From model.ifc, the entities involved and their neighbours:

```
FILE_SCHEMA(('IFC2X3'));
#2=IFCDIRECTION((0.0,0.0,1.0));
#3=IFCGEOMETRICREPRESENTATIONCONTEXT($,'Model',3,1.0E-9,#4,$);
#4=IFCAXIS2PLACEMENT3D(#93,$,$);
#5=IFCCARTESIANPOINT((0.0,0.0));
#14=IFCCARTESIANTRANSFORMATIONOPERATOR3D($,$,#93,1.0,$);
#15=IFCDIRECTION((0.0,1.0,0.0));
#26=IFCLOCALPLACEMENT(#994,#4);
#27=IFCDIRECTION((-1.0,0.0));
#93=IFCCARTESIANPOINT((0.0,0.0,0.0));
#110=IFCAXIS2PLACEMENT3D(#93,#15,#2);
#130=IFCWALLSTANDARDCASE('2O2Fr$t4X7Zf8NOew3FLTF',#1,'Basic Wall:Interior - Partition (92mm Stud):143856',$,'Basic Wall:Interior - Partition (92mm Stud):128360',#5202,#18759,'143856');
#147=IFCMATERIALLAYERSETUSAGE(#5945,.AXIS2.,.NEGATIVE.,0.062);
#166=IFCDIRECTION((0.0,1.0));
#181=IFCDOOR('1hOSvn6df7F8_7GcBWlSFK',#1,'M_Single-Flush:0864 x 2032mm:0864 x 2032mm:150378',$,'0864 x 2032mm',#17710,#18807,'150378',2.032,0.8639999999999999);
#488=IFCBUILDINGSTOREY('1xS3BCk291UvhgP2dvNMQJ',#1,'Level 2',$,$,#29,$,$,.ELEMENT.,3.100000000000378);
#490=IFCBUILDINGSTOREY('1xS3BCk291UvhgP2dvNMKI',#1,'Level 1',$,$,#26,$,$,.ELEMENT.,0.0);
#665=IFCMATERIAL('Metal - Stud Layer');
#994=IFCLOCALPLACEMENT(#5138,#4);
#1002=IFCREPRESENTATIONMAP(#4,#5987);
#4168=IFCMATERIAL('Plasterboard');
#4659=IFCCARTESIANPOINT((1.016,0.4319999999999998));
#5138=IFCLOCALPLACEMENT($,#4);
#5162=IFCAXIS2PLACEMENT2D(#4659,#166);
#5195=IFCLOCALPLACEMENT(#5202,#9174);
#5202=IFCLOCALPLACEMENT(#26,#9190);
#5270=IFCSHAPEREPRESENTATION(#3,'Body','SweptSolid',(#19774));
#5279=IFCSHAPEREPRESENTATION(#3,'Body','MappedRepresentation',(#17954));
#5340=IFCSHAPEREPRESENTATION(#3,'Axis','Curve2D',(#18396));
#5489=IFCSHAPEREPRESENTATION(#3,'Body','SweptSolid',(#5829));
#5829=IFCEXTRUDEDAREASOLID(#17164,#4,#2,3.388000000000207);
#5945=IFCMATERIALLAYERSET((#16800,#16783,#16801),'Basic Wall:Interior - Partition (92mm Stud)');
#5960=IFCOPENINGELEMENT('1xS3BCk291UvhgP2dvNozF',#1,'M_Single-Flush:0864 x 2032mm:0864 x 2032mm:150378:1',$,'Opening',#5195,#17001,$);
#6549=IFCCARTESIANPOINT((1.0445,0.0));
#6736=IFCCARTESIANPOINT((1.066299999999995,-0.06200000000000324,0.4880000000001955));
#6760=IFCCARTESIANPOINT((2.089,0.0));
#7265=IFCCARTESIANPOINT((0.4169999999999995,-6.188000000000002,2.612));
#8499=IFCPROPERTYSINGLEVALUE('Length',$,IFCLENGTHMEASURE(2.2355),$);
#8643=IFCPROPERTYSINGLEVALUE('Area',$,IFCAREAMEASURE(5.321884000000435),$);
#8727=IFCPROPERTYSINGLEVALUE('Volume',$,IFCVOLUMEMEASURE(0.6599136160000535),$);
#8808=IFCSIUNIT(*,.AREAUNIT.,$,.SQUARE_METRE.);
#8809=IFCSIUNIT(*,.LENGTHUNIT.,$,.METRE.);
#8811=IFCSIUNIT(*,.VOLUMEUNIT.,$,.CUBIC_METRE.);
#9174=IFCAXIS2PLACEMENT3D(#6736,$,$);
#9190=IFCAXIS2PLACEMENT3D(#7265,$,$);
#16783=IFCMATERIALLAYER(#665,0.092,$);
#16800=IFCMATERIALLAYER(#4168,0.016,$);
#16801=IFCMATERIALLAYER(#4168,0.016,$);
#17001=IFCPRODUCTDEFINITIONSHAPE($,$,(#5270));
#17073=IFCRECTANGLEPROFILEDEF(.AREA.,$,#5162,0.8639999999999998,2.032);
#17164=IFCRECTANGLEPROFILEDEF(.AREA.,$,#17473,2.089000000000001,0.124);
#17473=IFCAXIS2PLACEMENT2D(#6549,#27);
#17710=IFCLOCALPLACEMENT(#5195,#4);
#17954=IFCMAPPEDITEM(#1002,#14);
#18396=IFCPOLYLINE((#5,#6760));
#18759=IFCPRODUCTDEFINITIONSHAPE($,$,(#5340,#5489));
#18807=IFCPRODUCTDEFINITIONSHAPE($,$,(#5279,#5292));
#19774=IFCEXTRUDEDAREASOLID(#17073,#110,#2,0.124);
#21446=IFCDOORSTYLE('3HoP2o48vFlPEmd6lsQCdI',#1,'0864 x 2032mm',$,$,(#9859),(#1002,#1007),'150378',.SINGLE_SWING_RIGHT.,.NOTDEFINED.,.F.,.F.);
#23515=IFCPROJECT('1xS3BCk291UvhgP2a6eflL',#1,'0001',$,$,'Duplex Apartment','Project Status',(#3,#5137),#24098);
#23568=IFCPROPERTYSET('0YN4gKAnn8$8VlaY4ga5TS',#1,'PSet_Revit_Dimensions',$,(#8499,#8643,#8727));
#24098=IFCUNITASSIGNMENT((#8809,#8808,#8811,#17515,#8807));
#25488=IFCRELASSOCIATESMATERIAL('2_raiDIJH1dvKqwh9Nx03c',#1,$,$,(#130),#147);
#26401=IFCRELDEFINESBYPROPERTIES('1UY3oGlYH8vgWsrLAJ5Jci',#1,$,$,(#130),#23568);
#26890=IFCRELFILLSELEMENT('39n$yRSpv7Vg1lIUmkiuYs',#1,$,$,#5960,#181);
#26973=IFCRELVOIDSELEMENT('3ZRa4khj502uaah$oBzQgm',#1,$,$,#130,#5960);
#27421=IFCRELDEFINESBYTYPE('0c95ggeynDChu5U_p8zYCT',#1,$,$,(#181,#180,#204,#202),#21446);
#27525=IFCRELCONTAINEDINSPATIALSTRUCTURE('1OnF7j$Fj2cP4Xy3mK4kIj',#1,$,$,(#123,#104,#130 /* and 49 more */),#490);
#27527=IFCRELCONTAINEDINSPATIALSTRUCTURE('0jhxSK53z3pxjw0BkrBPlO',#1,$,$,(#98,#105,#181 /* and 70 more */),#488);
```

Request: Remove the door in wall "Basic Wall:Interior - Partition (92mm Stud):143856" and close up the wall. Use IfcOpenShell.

```python
import ifcopenshell
import ifcopenshell.api.feature
import ifcopenshell.api.pset
import ifcopenshell.api.root
import ifcopenshell.geom
import ifcopenshell.util.element
import ifcopenshell.util.shape
import ifcopenshell.util.unit

model = ifcopenshell.open("model.ifc")
area_scale = ifcopenshell.util.unit.calculate_unit_scale(model, "AREAUNIT")
volume_scale = ifcopenshell.util.unit.calculate_unit_scale(model, "VOLUMEUNIT")
settings = ifcopenshell.geom.settings()


def volume(element):
    """Net volume in cubic metres, openings subtracted."""
    shape = ifcopenshell.geom.create_shape(settings, element)
    return ifcopenshell.util.shape.get_volume(shape.geometry)


door = model.by_guid("1hOSvn6df7F8_7GcBWlSFK")
opening = door.FillsVoids[0].RelatingOpeningElement
wall = opening.VoidsElements[0].RelatingBuildingElement
before = volume(wall)

ifcopenshell.api.root.remove_product(model, product=door)
ifcopenshell.api.feature.remove_feature(model, feature=opening)

after = volume(wall)
thickness = 0.124  # wall thickness in metres

# Update the wall's stored quantities.
pset = model.by_id(ifcopenshell.util.element.get_pset(wall, "PSet_Revit_Dimensions", should_inherit=False)["id"])
ifcopenshell.api.pset.edit_pset(model, pset=pset, properties={
    "Area": model.create_entity("IfcAreaMeasure", after / thickness / area_scale),
    "Volume": model.create_entity("IfcVolumeMeasure", after / volume_scale),
})

print(f"wall volume {before:.3f} -> {after:.3f} m3")

model.write("model_updated.ifc")
```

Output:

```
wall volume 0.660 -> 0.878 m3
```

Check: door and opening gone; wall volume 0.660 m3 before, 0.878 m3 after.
